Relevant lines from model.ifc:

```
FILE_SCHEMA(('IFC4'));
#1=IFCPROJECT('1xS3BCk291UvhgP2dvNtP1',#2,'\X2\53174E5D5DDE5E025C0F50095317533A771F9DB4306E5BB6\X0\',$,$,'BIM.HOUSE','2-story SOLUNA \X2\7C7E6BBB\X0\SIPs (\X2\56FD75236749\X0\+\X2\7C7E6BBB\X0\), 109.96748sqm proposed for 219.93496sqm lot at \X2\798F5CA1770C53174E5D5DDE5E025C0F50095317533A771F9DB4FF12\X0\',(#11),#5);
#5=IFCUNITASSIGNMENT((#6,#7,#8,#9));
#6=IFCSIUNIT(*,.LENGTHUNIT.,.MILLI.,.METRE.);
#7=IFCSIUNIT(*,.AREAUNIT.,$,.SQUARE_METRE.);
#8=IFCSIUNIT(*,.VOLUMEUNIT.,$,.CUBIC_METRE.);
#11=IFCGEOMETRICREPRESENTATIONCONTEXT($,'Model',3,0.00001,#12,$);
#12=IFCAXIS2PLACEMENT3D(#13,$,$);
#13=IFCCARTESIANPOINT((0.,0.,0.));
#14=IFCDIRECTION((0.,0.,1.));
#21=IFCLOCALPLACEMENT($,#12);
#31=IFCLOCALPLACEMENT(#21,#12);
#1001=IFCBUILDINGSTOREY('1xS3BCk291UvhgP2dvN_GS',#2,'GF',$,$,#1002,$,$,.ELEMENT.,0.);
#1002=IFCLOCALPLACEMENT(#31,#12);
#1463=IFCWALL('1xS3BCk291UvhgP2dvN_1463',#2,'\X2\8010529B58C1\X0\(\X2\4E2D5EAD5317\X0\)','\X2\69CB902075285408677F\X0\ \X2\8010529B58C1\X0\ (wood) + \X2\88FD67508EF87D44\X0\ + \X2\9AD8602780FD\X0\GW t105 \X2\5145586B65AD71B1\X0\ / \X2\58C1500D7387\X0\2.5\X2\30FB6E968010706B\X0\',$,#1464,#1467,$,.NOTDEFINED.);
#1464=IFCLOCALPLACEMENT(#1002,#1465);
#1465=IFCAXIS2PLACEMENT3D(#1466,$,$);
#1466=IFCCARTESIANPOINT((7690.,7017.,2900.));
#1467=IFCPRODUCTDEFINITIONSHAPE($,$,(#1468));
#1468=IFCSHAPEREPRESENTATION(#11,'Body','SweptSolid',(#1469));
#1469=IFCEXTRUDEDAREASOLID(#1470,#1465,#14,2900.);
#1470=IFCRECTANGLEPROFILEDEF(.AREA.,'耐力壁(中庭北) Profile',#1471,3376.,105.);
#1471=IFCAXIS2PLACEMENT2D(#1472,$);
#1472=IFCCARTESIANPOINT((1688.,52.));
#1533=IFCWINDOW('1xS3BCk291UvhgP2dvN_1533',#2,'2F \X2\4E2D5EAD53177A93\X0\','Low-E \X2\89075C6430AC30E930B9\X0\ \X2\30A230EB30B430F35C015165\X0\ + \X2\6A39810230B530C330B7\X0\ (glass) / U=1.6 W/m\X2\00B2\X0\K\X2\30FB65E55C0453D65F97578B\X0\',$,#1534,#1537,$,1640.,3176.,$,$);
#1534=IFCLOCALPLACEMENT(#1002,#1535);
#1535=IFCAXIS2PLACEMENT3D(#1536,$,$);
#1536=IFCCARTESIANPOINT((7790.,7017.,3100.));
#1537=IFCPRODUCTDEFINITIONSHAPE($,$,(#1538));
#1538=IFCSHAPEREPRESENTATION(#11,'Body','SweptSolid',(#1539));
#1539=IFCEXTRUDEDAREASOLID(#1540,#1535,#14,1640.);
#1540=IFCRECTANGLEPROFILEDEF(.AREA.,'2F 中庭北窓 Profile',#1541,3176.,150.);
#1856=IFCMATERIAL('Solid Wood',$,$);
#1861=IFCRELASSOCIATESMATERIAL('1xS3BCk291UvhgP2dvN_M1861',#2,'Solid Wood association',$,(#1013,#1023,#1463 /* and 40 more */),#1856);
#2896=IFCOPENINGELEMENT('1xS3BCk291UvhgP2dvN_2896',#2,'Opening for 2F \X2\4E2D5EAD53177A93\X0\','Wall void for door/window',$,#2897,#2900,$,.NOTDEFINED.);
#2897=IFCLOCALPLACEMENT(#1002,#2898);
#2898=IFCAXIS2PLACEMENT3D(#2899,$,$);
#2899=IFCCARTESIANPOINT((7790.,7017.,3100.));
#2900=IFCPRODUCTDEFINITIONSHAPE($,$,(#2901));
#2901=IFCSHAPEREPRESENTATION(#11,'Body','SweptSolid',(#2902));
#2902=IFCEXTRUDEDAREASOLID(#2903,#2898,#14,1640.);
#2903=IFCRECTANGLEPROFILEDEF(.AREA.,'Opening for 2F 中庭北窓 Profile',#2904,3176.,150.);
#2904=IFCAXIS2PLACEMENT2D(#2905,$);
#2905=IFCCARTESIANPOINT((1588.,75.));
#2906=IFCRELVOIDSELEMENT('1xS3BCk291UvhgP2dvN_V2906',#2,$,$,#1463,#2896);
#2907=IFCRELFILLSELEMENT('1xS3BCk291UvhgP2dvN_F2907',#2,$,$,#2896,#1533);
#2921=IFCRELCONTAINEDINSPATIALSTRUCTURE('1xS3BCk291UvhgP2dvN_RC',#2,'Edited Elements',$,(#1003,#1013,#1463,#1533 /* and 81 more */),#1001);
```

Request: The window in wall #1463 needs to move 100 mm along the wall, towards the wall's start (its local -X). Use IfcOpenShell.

```python
import ifcopenshell
import ifcopenshell.api.geometry
import ifcopenshell.util.placement

model = ifcopenshell.open("model.ifc")

window = model.by_guid("1xS3BCk291UvhgP2dvN_1533")
opening = window.FillsVoids[0].RelatingOpeningElement
wall = opening.VoidsElements[0].RelatingBuildingElement

wall_matrix = ifcopenshell.util.placement.get_local_placement(wall.ObjectPlacement)
shift = wall_matrix[:3, 0] * -100.0
before = ifcopenshell.util.placement.get_local_placement(window.ObjectPlacement)[:3, 3].copy()

# The window is not placed relative to its opening, so move both.
for product in (opening, window):
    matrix = ifcopenshell.util.placement.get_local_placement(product.ObjectPlacement)
    matrix[:3, 3] += shift
    ifcopenshell.api.geometry.edit_object_placement(model, product=product, matrix=matrix, is_si=False)

after = ifcopenshell.util.placement.get_local_placement(window.ObjectPlacement)[:3, 3]
print("window moved by", (after - before).round(3) + 0.0)

model.write("model_rev.ifc")
```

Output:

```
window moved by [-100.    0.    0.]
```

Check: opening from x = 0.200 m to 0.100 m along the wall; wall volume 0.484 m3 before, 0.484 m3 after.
